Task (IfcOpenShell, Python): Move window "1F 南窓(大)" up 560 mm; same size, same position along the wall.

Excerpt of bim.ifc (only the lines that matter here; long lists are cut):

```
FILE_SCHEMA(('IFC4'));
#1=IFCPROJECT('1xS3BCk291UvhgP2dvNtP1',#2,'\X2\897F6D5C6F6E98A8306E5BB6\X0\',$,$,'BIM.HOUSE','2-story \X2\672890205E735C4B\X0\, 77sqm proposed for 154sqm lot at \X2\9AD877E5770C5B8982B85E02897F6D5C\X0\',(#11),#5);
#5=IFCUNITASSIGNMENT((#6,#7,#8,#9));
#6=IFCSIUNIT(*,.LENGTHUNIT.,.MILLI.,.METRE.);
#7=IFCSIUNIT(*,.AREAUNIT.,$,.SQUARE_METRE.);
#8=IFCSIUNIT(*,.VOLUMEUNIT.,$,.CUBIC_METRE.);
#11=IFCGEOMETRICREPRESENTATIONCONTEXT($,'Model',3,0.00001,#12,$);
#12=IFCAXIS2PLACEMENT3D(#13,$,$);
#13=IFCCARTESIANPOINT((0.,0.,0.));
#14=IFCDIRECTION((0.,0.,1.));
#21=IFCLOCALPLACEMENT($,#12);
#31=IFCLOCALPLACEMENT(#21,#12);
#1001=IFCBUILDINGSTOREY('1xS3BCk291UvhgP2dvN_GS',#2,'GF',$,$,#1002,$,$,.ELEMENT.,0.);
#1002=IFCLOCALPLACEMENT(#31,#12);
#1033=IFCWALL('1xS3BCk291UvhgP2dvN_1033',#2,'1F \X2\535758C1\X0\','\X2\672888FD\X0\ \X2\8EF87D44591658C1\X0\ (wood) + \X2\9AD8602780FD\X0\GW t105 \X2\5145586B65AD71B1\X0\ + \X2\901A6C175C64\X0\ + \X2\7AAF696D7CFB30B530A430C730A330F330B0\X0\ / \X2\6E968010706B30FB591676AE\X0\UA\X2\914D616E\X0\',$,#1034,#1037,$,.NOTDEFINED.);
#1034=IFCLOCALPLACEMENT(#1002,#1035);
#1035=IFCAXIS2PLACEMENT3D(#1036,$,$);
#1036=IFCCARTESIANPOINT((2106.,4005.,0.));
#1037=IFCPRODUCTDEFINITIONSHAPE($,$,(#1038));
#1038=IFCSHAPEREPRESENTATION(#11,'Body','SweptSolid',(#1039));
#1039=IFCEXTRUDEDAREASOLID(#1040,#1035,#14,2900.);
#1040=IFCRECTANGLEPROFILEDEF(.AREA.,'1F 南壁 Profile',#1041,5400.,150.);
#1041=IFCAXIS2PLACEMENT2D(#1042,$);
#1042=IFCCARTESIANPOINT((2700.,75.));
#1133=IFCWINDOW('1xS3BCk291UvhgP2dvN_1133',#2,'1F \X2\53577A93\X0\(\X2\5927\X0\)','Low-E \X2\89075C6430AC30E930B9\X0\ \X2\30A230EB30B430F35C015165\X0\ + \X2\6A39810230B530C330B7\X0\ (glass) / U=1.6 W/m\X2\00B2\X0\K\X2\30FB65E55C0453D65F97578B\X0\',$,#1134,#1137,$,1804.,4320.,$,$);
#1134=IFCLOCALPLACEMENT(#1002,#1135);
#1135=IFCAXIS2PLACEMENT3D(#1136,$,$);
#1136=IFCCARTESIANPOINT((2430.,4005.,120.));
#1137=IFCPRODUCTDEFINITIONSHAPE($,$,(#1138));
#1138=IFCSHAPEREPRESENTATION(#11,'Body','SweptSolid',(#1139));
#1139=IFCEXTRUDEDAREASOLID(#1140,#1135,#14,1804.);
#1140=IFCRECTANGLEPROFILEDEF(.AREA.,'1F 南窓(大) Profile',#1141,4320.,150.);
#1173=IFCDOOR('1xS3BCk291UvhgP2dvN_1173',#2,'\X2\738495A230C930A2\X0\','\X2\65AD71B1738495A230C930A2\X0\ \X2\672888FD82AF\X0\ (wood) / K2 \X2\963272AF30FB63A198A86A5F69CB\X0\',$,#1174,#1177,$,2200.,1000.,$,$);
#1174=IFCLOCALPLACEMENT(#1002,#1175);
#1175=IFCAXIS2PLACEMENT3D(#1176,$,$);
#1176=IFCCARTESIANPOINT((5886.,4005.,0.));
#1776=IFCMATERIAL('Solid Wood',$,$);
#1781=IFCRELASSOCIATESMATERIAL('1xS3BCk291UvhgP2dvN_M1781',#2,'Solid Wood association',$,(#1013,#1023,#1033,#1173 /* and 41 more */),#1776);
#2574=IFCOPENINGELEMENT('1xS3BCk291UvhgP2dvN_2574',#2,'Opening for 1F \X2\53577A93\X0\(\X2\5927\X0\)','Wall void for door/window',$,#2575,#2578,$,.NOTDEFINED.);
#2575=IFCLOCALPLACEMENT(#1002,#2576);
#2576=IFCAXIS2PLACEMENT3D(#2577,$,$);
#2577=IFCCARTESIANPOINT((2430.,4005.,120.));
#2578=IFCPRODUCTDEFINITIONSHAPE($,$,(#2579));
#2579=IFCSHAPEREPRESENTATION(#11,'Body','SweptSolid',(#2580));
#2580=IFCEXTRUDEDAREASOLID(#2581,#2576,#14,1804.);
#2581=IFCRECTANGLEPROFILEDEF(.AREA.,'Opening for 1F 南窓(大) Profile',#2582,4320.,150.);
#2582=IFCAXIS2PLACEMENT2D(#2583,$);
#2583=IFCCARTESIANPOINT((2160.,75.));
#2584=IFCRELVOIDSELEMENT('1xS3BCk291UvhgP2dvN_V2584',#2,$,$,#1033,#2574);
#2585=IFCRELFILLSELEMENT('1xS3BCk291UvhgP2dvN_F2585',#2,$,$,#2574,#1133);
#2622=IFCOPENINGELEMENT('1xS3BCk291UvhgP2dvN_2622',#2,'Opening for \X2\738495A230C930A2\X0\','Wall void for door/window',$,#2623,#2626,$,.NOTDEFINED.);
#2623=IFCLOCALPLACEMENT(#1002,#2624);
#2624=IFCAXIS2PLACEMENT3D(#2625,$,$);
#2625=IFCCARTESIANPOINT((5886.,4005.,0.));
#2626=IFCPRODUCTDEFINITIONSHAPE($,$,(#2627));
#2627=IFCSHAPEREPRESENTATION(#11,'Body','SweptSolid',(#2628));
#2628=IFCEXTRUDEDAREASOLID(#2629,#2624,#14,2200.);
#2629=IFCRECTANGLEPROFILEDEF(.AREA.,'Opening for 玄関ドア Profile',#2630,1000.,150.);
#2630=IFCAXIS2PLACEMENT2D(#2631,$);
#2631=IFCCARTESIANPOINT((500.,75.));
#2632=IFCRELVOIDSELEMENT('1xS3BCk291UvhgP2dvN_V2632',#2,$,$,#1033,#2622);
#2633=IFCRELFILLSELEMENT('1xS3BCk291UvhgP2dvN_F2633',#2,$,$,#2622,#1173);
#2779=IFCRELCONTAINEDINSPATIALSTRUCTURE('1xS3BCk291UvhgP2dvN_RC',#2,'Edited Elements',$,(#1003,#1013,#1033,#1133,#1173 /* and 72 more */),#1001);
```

```python
import numpy as np
import ifcopenshell
import ifcopenshell.api.geometry
import ifcopenshell.util.placement
import ifcopenshell.util.unit

model = ifcopenshell.open("bim.ifc")
unit_scale = ifcopenshell.util.unit.calculate_unit_scale(model)

window = model.by_id(1133)
opening = window.FillsVoids[0].RelatingOpeningElement
dz = 0.56 / unit_scale

shift = np.array([0.0, 0.0, dz])
# The window is not placed relative to its opening, so move both.
for product in (opening, window):
    matrix = ifcopenshell.util.placement.get_local_placement(product.ObjectPlacement)
    matrix[:3, 3] += shift
    ifcopenshell.api.geometry.edit_object_placement(model, product=product, matrix=matrix, is_si=False)

print(f"moved by {dz * unit_scale:+.3f} m")

model.write("bim-out.ifc")
```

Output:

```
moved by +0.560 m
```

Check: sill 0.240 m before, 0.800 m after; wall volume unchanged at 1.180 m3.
